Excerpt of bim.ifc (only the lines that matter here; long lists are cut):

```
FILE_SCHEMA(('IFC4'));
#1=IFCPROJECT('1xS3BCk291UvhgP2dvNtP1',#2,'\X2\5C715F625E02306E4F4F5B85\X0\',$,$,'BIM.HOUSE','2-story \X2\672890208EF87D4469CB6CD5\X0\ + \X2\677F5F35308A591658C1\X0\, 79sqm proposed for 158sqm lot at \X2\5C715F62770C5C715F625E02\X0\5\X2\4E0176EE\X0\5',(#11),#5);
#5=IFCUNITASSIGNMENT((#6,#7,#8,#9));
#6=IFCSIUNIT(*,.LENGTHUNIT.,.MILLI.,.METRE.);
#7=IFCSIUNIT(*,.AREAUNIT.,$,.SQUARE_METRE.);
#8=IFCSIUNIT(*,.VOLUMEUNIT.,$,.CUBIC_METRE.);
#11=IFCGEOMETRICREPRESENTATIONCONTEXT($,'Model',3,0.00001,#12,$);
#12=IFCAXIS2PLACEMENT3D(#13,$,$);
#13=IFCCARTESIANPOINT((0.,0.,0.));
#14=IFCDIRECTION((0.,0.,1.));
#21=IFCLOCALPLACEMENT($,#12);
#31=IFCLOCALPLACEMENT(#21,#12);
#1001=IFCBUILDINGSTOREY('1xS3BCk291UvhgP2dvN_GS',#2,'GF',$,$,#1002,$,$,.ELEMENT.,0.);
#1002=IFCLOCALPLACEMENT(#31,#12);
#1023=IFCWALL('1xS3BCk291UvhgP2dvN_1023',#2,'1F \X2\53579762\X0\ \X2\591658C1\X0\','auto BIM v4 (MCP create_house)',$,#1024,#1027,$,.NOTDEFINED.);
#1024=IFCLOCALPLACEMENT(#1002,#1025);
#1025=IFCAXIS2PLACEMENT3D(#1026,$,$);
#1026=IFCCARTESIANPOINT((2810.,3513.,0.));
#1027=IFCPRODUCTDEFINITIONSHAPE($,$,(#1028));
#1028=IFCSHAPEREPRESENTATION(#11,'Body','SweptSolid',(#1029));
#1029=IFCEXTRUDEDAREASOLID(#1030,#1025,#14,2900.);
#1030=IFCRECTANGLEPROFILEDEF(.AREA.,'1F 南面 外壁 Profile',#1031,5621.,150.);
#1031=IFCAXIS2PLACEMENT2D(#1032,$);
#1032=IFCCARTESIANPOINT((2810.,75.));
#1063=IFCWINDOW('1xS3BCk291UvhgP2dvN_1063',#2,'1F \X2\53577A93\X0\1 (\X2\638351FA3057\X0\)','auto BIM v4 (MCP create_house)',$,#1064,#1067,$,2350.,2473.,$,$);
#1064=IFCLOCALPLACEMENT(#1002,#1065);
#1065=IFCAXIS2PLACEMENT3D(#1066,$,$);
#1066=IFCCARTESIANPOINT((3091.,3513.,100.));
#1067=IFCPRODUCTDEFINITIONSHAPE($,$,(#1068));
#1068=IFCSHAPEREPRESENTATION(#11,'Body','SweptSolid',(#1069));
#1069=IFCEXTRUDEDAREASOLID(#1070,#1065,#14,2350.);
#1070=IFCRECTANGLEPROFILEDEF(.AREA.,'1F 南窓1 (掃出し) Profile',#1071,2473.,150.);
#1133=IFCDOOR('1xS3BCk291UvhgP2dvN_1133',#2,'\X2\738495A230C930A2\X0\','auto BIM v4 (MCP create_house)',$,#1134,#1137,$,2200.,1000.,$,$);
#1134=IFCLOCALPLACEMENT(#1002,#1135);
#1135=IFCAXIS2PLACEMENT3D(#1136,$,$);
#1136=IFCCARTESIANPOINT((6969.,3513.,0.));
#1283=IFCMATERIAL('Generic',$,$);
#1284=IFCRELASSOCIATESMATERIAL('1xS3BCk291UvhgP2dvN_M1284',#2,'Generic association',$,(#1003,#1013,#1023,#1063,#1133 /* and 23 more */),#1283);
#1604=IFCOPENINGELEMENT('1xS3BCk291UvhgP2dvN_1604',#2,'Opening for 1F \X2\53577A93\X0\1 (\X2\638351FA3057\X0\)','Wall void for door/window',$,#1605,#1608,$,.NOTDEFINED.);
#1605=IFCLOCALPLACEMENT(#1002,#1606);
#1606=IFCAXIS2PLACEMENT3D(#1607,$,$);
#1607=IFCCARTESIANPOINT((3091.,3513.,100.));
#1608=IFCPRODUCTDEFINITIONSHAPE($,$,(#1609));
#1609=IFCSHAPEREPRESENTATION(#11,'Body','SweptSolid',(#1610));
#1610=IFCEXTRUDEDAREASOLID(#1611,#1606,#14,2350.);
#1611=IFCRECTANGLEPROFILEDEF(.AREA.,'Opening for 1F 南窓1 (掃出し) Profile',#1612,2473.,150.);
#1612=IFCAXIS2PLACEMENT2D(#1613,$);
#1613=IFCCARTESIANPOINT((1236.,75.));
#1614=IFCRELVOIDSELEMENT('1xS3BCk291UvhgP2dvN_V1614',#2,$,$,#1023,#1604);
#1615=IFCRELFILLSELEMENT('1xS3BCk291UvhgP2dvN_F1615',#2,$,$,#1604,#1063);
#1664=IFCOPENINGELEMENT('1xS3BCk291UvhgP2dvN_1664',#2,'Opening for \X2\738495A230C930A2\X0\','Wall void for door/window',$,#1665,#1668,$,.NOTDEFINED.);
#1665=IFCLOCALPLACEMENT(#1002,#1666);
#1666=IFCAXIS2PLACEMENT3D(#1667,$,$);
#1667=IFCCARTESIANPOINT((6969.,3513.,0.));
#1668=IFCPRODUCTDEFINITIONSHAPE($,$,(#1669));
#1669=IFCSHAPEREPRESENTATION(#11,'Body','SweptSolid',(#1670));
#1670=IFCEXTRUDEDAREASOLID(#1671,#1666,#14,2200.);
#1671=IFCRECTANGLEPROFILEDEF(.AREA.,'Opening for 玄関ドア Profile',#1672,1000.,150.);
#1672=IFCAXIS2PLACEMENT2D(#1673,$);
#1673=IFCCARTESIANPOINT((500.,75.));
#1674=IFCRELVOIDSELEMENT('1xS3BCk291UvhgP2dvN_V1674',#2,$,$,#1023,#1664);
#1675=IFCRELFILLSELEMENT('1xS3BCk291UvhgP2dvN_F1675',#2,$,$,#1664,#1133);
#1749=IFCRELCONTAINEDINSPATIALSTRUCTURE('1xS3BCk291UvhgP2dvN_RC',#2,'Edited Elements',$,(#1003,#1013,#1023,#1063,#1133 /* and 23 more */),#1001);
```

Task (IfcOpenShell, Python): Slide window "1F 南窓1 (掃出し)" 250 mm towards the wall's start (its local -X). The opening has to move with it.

```python
import ifcopenshell
import ifcopenshell.api.geometry
import ifcopenshell.util.placement
import ifcopenshell.util.unit

model = ifcopenshell.open("bim.ifc")
unit_scale = ifcopenshell.util.unit.calculate_unit_scale(model)

window = model.by_guid("1xS3BCk291UvhgP2dvN_1063")
opening = window.FillsVoids[0].RelatingOpeningElement
wall = opening.VoidsElements[0].RelatingBuildingElement

wall_matrix = ifcopenshell.util.placement.get_local_placement(wall.ObjectPlacement)
shift = wall_matrix[:3, 0] * -0.25 / unit_scale
before = ifcopenshell.util.placement.get_local_placement(window.ObjectPlacement)[:3, 3].copy()

# The window is not placed relative to its opening, so move both.
for product in (opening, window):
    matrix = ifcopenshell.util.placement.get_local_placement(product.ObjectPlacement)
    matrix[:3, 3] += shift
    ifcopenshell.api.geometry.edit_object_placement(model, product=product, matrix=matrix, is_si=False)

after = ifcopenshell.util.placement.get_local_placement(window.ObjectPlacement)[:3, 3]
print("window moved by", (after - before).round(3) + 0.0)

model.write("bim_updated.ifc")
```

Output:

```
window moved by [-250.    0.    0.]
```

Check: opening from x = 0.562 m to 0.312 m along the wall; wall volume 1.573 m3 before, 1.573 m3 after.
